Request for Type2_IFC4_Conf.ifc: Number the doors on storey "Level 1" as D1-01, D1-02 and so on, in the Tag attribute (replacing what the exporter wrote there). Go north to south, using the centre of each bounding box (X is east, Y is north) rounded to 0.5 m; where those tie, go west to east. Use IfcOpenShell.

First a look at what the model holds.

```python
import ifcopenshell
import ifcopenshell.util.element
import ifcopenshell.util.placement

model = ifcopenshell.open("Type2_IFC4_Conf.ifc")
print(model.schema)
storey = next(s for s in model.by_type("IfcBuildingStorey") if s.Name == "Level 1")
doors = [e for e in ifcopenshell.util.element.get_decomposition(storey) if e.is_a("IfcDoor")]
for e in sorted(doors, key=lambda e: e.id()):
    origin = ifcopenshell.util.placement.get_local_placement(e.ObjectPlacement)[:3, 3]
    print(e.id(), e.Tag, e.Name, origin.round(2) + 0.0, sep=" | ")
```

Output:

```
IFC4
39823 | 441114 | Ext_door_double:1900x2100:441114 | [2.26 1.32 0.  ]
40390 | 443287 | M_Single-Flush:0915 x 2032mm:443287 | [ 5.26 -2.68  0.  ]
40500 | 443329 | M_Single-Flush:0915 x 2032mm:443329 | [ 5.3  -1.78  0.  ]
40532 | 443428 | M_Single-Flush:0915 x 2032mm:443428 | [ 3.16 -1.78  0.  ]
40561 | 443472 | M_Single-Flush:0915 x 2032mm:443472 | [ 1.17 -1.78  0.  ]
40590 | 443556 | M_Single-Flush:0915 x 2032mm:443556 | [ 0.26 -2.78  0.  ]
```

```python
import ifcopenshell
import ifcopenshell.geom
import ifcopenshell.util.element
import ifcopenshell.util.shape

model = ifcopenshell.open("Type2_IFC4_Conf.ifc")
settings = ifcopenshell.geom.settings()
settings.set("use-world-coords", True)


def centre(element):
    shape = ifcopenshell.geom.create_shape(settings, element)
    return ifcopenshell.util.shape.get_bbox_centroid(shape.geometry)


storey = next(s for s in model.by_type("IfcBuildingStorey") if s.Name == "Level 1")
doors = [e for e in ifcopenshell.util.element.get_decomposition(storey) if e.is_a("IfcDoor")]

# Insertion points can sit at a corner or the storey origin, so sort by the geometry (in metres).
centres = {e: centre(e) for e in doors}
doors.sort(key=lambda e: (-round(centres[e][1] / 0.5), centres[e][0]))

for i, e in enumerate(doors, start=1):
    number = f"D1-{i:02d}"
    e.Tag = number
    print(e.id(), number)

model.write("Type2_IFC4_Conf_rev.ifc")
```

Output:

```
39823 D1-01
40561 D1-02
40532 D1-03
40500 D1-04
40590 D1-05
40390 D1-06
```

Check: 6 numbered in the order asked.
